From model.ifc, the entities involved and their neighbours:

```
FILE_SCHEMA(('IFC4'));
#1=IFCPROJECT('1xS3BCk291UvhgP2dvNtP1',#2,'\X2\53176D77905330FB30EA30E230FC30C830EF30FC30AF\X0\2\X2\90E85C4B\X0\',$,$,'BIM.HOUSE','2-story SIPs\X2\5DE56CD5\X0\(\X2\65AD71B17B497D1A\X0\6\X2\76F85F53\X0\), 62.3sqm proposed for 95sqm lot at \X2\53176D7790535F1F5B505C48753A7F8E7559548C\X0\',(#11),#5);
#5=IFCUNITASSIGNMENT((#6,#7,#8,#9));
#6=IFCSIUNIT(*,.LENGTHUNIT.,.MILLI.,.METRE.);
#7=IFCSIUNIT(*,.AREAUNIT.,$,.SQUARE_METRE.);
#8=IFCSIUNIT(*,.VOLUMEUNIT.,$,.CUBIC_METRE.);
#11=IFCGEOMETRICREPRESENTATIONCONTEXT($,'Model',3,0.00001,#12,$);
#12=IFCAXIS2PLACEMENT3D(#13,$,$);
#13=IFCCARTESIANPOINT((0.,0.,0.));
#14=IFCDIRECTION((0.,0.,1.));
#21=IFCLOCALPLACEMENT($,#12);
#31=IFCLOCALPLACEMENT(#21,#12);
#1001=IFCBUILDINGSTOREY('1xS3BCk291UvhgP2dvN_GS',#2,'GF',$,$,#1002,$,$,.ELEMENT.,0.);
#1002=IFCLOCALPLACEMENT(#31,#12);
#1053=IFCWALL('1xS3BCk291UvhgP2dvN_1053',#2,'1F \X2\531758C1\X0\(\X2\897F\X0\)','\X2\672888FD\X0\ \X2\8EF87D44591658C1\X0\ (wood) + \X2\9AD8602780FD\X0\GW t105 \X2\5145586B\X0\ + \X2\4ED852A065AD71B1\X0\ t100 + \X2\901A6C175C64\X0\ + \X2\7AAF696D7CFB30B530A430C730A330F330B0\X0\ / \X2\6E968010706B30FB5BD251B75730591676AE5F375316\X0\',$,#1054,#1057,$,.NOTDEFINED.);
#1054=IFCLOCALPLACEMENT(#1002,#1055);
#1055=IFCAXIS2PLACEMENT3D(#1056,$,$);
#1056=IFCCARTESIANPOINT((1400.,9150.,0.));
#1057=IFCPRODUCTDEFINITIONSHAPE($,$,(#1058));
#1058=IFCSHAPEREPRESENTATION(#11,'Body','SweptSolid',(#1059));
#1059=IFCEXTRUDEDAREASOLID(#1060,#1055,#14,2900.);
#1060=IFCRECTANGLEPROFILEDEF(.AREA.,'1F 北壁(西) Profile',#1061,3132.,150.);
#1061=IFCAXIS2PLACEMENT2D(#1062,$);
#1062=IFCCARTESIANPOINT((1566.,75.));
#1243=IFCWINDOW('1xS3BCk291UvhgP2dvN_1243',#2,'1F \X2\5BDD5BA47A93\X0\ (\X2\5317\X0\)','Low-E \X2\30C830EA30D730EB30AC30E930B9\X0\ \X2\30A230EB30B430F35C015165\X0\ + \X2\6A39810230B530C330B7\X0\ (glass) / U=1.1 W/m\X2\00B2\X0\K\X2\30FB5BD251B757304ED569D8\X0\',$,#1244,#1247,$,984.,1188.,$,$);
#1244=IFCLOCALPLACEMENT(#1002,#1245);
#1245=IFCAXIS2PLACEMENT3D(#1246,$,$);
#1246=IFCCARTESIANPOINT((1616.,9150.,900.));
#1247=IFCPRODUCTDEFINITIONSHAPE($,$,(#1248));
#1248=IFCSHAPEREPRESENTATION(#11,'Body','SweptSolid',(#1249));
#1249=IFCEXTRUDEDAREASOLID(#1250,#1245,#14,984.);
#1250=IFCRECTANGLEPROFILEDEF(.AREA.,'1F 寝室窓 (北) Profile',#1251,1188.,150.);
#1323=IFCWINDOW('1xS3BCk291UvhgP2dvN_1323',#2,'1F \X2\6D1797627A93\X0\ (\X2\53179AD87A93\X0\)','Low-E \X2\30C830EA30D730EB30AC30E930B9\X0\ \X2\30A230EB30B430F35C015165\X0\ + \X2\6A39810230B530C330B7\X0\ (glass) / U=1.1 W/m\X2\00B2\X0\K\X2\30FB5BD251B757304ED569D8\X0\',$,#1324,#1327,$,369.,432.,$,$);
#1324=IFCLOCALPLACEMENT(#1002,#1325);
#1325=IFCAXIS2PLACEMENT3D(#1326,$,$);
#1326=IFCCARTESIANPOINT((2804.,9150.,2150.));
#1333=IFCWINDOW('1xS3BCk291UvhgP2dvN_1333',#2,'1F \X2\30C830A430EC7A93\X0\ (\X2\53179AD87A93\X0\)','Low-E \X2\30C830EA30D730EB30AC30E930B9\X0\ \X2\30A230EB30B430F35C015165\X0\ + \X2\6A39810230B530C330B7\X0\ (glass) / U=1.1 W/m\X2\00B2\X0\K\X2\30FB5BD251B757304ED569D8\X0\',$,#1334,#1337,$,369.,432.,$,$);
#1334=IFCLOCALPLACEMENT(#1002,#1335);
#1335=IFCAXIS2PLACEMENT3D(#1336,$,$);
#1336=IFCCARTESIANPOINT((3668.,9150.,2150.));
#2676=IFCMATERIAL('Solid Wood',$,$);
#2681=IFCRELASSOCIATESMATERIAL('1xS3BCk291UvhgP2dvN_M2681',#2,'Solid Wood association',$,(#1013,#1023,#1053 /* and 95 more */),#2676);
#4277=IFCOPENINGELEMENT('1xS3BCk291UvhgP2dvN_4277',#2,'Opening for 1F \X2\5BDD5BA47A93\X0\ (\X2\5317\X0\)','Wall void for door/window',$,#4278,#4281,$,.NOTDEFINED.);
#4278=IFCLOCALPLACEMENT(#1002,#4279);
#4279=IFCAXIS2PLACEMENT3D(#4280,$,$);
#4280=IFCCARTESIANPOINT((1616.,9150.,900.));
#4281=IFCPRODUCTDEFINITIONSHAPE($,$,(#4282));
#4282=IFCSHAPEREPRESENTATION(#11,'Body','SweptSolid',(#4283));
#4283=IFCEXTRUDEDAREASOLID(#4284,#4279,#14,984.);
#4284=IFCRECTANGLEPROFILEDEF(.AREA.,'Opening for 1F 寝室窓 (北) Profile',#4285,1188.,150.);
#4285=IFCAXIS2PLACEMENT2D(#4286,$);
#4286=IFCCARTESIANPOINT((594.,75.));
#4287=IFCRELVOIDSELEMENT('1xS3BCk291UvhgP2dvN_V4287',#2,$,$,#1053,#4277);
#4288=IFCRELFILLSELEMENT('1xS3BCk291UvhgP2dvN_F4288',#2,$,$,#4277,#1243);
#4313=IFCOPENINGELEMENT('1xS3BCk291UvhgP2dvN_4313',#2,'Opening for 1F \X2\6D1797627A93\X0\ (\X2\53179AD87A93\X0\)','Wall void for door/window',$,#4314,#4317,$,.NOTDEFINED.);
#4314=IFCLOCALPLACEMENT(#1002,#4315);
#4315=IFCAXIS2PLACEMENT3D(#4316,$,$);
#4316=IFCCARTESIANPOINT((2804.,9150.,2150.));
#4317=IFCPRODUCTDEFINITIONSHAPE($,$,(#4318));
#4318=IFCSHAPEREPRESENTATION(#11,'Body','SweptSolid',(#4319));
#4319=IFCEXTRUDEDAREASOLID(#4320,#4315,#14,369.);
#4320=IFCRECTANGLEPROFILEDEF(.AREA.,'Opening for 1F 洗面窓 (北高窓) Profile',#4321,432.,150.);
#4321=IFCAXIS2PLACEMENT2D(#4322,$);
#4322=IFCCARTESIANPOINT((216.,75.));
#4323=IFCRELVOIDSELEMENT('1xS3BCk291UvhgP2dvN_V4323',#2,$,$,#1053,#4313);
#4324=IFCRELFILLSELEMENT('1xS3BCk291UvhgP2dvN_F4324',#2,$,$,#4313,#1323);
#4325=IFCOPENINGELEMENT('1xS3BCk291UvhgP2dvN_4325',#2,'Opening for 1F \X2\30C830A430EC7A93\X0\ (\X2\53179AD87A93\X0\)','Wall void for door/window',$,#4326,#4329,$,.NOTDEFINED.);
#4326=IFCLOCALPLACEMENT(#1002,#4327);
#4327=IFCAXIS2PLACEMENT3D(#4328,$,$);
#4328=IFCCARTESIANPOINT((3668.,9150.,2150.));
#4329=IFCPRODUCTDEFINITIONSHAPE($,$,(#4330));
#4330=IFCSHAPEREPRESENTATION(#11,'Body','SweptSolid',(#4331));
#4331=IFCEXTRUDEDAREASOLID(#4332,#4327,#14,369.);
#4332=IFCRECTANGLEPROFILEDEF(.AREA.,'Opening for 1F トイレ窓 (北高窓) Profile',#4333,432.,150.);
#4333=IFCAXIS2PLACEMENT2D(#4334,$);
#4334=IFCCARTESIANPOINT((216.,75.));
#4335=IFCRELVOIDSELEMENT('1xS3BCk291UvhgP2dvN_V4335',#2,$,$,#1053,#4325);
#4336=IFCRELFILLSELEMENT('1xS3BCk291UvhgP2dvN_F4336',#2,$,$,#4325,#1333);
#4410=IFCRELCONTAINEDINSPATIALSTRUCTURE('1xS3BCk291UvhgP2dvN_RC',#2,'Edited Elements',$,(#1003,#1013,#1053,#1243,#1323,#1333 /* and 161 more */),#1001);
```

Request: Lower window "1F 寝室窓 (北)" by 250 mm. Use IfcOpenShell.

```python
import numpy as np
import ifcopenshell
import ifcopenshell.api.geometry
import ifcopenshell.util.placement
import ifcopenshell.util.unit

model = ifcopenshell.open("model.ifc")
unit_scale = ifcopenshell.util.unit.calculate_unit_scale(model)

window = model.by_guid("1xS3BCk291UvhgP2dvN_1243")
opening = window.FillsVoids[0].RelatingOpeningElement
dz = -250.0

shift = np.array([0.0, 0.0, dz])
# The window is not placed relative to its opening, so move both.
for product in (opening, window):
    matrix = ifcopenshell.util.placement.get_local_placement(product.ObjectPlacement)
    matrix[:3, 3] += shift
    ifcopenshell.api.geometry.edit_object_placement(model, product=product, matrix=matrix, is_si=False)

print(f"moved by {dz * unit_scale:+.3f} m")

model.write("model_updated.ifc")
```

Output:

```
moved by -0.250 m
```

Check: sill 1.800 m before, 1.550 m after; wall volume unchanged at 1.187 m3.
